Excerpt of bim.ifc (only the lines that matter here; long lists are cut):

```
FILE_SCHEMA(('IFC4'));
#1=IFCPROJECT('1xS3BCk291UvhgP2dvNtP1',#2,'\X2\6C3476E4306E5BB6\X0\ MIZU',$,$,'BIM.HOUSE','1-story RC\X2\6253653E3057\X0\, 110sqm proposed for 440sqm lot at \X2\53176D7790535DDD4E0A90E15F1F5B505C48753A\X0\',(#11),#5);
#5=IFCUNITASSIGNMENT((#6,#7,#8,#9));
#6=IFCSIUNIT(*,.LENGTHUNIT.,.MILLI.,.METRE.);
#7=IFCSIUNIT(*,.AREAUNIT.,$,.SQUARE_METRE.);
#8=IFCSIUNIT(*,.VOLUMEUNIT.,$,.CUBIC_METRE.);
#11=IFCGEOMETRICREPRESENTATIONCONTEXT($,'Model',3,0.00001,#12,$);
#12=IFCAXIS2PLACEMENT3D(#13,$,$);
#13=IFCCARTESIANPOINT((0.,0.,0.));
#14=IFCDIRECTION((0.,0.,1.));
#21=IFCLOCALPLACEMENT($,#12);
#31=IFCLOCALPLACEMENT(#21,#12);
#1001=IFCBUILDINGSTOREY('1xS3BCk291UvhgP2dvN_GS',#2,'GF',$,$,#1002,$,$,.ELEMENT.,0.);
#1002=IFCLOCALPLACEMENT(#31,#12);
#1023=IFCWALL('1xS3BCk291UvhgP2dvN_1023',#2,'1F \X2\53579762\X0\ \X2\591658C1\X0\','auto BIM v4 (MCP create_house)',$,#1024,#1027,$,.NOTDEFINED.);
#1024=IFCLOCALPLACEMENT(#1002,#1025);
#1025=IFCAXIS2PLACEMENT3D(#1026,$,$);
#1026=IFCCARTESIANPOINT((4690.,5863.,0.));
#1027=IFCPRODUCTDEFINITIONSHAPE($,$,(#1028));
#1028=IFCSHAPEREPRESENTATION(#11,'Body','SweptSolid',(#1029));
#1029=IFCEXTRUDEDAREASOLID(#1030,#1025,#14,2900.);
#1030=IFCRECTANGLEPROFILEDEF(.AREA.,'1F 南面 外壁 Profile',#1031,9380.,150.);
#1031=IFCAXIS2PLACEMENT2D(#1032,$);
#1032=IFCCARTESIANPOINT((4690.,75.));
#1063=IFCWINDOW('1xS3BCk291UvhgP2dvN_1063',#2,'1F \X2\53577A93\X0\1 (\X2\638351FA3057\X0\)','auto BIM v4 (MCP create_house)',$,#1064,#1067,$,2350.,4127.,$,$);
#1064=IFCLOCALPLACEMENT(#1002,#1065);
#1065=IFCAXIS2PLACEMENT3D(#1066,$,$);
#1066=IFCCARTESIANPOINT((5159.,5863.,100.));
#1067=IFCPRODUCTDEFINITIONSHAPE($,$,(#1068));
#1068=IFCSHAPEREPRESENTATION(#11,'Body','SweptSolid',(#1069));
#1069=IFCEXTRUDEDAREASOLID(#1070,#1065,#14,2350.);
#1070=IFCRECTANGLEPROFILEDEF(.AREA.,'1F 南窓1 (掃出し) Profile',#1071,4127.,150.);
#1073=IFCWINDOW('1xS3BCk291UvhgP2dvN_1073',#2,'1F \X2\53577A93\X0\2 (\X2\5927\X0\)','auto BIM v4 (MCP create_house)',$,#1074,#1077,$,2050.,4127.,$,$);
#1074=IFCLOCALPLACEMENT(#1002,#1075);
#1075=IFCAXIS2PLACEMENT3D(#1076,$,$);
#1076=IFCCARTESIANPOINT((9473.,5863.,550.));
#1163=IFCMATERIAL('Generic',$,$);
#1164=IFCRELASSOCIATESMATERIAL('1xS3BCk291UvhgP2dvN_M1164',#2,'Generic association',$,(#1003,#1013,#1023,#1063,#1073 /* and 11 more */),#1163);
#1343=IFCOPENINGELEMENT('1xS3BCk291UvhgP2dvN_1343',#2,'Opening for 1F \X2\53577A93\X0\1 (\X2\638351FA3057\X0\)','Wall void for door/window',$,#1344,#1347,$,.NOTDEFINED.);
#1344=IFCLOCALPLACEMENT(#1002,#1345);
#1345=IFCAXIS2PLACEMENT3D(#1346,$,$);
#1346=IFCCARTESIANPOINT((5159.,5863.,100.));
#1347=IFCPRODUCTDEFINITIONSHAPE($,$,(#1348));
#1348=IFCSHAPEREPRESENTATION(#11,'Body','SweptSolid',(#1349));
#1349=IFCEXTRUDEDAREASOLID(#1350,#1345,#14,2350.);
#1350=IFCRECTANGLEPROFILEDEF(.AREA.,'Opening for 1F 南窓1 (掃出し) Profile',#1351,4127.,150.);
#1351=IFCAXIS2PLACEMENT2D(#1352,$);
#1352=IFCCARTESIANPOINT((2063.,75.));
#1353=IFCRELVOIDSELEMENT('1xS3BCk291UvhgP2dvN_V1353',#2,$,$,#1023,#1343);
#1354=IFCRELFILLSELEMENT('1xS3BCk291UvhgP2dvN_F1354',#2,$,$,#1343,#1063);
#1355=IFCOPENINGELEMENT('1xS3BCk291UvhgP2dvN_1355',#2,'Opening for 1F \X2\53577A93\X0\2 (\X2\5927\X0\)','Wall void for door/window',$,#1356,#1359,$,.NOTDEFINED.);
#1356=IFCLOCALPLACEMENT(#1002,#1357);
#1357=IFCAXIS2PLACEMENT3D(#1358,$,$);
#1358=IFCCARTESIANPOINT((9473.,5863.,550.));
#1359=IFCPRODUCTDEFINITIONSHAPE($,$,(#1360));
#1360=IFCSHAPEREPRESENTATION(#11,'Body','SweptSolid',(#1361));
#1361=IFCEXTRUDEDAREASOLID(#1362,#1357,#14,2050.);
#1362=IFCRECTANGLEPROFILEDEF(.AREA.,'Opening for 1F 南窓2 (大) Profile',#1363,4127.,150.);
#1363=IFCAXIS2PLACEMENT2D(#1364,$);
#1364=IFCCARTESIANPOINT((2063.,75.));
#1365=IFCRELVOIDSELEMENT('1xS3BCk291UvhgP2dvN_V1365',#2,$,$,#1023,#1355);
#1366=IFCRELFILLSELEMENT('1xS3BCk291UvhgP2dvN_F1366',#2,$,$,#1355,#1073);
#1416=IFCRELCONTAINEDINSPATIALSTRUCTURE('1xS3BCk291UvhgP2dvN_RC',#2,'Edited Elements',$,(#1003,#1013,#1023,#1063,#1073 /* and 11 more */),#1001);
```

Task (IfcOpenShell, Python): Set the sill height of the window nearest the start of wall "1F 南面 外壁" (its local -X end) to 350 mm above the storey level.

```python
import numpy as np
import ifcopenshell
import ifcopenshell.api.geometry
import ifcopenshell.geom
import ifcopenshell.util.element
import ifcopenshell.util.placement
import ifcopenshell.util.shape
import ifcopenshell.util.unit

model = ifcopenshell.open("bim.ifc")
unit_scale = ifcopenshell.util.unit.calculate_unit_scale(model)

window = model.by_id(1063)
opening = window.FillsVoids[0].RelatingOpeningElement
storey = ifcopenshell.util.element.get_container(window, ifc_class="IfcBuildingStorey")
level = ifcopenshell.util.placement.get_local_placement(storey.ObjectPlacement)[2, 3]

# The opening's origin need not be at the sill, so measure its lowest point.
shape = ifcopenshell.geom.create_shape(ifcopenshell.geom.settings(), opening)
bottom = ifcopenshell.util.shape.get_shape_bottom_elevation(shape, shape.geometry) / unit_scale
dz = level + 350.0 - bottom

shift = np.array([0.0, 0.0, dz])
# The window is not placed relative to its opening, so move both.
for product in (opening, window):
    matrix = ifcopenshell.util.placement.get_local_placement(product.ObjectPlacement)
    matrix[:3, 3] += shift
    ifcopenshell.api.geometry.edit_object_placement(model, product=product, matrix=matrix, is_si=False)

print(f"moved by {dz * unit_scale:+.3f} m")

model.write("bim_v2.ifc")
```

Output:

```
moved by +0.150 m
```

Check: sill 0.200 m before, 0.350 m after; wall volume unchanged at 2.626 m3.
